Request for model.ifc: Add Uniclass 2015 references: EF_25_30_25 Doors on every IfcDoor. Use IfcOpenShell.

First a look at what the model holds.

```python
import ifcopenshell

model = ifcopenshell.open("model.ifc")
print(model.schema)
print("classifications:", [c.Name for c in model.by_type("IfcClassification")])
for ifc_class in ("IfcDoor", "IfcRoof", "IfcStair", "IfcWall", "IfcWindow"):
    print(ifc_class, len(model.by_type(ifc_class)))
```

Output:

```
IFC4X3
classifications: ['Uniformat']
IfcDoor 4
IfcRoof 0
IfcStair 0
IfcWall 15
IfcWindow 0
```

```python
import ifcopenshell
import ifcopenshell.api.classification

model = ifcopenshell.open("model.ifc")

system = ifcopenshell.api.classification.add_classification(model, classification="Uniclass 2015")

codes = {
    "IfcDoor": ("EF_25_30_25", "Doors"),
}
for ifc_class, (code, name) in codes.items():
    products = model.by_type(ifc_class)
    ifcopenshell.api.classification.add_reference(
        model, products=products, classification=system, identification=code, name=name
    )
    print(code, len(products))

model.write("model_v2.ifc")
```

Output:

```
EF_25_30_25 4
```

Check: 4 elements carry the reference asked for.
